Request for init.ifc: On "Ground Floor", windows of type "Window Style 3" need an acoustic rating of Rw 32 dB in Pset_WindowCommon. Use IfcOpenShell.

First a look at what the model holds.

```python
import ifcopenshell
import ifcopenshell.util.element

model = ifcopenshell.open("init.ifc")
print(model.schema)
storey = next(s for s in model.by_type("IfcBuildingStorey") if s.Name == "Ground Floor")
windows = [e for e in ifcopenshell.util.element.get_decomposition(storey) if e.is_a("IfcWindow")]
seen = {}
for e in windows:
    element_type = ifcopenshell.util.element.get_type(e)
    key = (element_type.Name if element_type != e and element_type else None, ifcopenshell.util.element.get_pset(e, "Pset_WindowCommon", "AcousticRating"))
    seen[key] = seen.get(key, 0) + 1
for (name, value), count in sorted(seen.items(), key=str):
    print(count, "x", name, "|", value)
```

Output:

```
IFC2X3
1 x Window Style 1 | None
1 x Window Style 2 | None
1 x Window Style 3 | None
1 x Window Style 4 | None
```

```python
import ifcopenshell
import ifcopenshell.api.pset
import ifcopenshell.util.element

model = ifcopenshell.open("init.ifc")

storey = next(s for s in model.by_type("IfcBuildingStorey") if s.Name == "Ground Floor")
windows = [e for e in ifcopenshell.util.element.get_decomposition(storey) if e.is_a("IfcWindow")]

count = 0
for e in windows:
    element_type = ifcopenshell.util.element.get_type(e)
    if element_type in (None, e) or element_type.Name != "Window Style 3":
        continue
    # add_pset returns the element's existing set when there is one.
    pset = ifcopenshell.api.pset.add_pset(model, product=e, name="Pset_WindowCommon")
    ifcopenshell.api.pset.edit_pset(model, pset=pset, properties={"AcousticRating": "Rw 32 dB"})
    count += 1

print(count, "windows updated")

model.write("init_rev.ifc")
```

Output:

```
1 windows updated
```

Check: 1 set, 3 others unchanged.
